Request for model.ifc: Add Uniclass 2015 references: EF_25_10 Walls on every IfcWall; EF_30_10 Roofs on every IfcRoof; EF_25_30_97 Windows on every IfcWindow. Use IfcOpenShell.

First a look at what the model holds.

```python
import ifcopenshell

model = ifcopenshell.open("model.ifc")
print(model.schema)
print("classifications:", [c.Name for c in model.by_type("IfcClassification")])
for ifc_class in ("IfcDoor", "IfcRoof", "IfcStair", "IfcWall", "IfcWindow"):
    print(ifc_class, len(model.by_type(ifc_class)))
```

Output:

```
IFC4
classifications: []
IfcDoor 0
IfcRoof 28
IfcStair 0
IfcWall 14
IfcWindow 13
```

```python
import ifcopenshell
import ifcopenshell.api.classification

model = ifcopenshell.open("model.ifc")

system = ifcopenshell.api.classification.add_classification(model, classification="Uniclass 2015")

codes = {
    "IfcWall": ("EF_25_10", "Walls"),
    "IfcRoof": ("EF_30_10", "Roofs"),
    "IfcWindow": ("EF_25_30_97", "Windows"),
}
for ifc_class, (code, name) in codes.items():
    products = model.by_type(ifc_class)
    ifcopenshell.api.classification.add_reference(
        model, products=products, classification=system, identification=code, name=name
    )
    print(code, len(products))

model.write("model_updated.ifc")
```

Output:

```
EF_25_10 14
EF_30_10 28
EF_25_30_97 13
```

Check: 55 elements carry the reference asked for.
